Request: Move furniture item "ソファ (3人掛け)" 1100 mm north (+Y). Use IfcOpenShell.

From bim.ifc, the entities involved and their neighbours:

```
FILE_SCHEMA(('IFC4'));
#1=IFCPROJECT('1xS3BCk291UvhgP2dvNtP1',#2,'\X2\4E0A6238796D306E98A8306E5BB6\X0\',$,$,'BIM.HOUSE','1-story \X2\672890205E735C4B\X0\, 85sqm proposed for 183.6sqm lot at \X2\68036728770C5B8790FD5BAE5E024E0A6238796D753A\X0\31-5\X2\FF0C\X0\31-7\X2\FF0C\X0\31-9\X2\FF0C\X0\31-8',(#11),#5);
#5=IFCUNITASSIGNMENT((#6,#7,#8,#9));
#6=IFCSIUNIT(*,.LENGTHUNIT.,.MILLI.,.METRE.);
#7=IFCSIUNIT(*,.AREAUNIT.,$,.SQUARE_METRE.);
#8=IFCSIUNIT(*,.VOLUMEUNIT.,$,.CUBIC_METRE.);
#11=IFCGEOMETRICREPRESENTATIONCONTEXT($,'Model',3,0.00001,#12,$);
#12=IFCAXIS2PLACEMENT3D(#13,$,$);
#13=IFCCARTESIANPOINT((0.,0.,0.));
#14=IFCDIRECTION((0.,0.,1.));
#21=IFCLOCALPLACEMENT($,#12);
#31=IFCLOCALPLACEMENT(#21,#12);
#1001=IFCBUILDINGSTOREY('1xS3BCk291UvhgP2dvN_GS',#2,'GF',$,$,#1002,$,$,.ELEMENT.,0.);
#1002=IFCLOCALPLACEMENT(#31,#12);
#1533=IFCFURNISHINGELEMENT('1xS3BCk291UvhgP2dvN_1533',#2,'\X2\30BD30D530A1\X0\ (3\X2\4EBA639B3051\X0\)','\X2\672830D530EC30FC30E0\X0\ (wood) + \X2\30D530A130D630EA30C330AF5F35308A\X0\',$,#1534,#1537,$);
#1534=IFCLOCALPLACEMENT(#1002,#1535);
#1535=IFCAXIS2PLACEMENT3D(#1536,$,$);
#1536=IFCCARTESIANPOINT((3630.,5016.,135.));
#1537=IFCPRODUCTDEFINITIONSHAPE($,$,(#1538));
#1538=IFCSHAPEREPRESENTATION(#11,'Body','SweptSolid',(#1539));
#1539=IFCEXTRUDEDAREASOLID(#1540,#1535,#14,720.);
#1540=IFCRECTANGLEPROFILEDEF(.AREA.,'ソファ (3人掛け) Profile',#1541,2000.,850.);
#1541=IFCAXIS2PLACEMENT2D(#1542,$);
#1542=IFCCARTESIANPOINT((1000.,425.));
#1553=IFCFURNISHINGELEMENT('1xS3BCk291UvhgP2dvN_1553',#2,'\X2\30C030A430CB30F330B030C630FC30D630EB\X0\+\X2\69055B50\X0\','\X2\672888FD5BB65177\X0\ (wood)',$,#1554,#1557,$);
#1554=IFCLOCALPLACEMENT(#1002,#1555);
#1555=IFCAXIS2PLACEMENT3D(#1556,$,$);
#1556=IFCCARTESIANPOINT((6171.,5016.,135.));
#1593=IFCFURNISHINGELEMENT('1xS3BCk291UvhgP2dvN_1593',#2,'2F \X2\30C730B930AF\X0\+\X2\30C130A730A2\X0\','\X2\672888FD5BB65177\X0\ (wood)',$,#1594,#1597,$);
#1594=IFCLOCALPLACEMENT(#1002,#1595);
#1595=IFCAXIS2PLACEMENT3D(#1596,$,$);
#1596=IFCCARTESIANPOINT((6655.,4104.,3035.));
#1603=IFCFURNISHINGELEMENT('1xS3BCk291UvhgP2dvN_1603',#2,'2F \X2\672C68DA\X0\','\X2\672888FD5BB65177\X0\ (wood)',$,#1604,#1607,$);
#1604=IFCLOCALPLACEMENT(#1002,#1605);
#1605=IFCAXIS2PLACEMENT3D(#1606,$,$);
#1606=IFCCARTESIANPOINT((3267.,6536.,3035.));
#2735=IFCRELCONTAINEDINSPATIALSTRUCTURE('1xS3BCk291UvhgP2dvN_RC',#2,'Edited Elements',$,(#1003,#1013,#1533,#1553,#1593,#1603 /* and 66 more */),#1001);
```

```python
import ifcopenshell
import ifcopenshell.api.geometry
import ifcopenshell.util.placement
import ifcopenshell.util.unit

model = ifcopenshell.open("bim.ifc")
unit_scale = ifcopenshell.util.unit.calculate_unit_scale(model)

item = model.by_id(1533)
matrix = ifcopenshell.util.placement.get_local_placement(item.ObjectPlacement)
matrix[1, 3] += 1.1 / unit_scale
ifcopenshell.api.geometry.edit_object_placement(model, product=item, matrix=matrix, is_si=False)

print(ifcopenshell.util.placement.get_local_placement(item.ObjectPlacement).round(3) + 0.0)

model.write("bim_rev.ifc")
```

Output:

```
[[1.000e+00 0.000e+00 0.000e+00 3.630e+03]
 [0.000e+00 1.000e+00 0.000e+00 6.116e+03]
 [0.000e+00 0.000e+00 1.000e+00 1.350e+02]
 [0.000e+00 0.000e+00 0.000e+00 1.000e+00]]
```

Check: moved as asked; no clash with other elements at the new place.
